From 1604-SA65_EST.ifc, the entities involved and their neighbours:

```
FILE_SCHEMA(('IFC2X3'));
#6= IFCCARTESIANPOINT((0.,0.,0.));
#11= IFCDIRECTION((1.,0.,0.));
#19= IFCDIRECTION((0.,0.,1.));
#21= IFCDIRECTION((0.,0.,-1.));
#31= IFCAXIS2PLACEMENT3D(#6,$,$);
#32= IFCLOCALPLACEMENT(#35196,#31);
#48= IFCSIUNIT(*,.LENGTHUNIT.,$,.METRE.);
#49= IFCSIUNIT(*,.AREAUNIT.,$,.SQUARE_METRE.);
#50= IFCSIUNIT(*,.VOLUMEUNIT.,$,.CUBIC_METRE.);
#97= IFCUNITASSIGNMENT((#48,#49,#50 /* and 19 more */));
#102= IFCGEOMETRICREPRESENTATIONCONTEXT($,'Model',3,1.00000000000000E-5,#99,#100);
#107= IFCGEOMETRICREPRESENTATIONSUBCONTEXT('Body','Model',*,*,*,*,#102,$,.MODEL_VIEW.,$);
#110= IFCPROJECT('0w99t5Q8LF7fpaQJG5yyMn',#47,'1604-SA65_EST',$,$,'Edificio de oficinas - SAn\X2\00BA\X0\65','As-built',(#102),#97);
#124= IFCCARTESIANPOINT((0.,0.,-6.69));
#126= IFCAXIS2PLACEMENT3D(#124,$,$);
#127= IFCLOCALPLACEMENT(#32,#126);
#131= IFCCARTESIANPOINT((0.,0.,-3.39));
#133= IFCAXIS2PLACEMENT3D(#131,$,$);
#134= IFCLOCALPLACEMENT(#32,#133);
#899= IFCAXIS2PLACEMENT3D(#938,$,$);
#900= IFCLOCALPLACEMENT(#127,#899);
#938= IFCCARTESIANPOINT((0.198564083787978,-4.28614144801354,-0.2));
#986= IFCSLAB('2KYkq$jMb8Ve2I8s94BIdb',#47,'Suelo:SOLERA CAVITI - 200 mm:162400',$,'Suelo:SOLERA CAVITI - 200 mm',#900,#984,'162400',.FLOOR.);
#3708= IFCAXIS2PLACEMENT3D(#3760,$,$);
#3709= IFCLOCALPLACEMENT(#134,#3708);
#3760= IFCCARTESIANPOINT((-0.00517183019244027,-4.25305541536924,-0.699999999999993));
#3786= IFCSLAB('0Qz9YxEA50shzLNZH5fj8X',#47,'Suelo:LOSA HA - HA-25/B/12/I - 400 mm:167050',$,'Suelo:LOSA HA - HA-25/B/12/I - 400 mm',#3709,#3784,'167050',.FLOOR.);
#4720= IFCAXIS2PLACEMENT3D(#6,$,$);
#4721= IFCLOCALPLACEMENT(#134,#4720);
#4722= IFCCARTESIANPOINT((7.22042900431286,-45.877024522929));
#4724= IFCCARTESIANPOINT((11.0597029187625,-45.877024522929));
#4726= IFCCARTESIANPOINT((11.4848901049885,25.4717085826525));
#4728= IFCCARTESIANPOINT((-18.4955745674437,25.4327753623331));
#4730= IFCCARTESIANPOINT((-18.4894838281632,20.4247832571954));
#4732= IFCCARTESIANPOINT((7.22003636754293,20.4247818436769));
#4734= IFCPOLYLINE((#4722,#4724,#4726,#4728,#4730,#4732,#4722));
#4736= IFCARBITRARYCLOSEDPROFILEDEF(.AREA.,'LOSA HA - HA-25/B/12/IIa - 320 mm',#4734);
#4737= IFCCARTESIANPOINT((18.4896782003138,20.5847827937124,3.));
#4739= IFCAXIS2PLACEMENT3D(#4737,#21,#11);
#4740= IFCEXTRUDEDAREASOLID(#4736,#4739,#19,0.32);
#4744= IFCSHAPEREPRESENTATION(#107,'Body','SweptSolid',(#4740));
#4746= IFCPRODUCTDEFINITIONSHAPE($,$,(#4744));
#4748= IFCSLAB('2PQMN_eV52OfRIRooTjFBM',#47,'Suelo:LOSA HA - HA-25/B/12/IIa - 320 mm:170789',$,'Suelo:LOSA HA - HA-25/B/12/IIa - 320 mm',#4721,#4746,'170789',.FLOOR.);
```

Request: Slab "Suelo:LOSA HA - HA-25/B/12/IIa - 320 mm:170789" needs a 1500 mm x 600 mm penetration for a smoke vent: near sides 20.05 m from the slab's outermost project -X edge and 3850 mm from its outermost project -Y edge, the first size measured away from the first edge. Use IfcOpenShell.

```python
import numpy as np
import ifcopenshell
import ifcopenshell.api.feature
import ifcopenshell.api.geometry
import ifcopenshell.api.root
import ifcopenshell.geom
import ifcopenshell.util.placement
import ifcopenshell.util.representation
import ifcopenshell.util.shape
import ifcopenshell.util.unit

model = ifcopenshell.open("1604-SA65_EST.ifc")
unit_scale = ifcopenshell.util.unit.calculate_unit_scale(model)
settings = ifcopenshell.geom.settings()


def volume(element):
    """Net volume in cubic metres, openings subtracted."""
    shape = ifcopenshell.geom.create_shape(settings, element)
    return ifcopenshell.util.shape.get_volume(shape.geometry)


slab = model.by_guid("2PQMN_eV52OfRIRooTjFBM")
before = volume(slab)

# Extent in the slab's own axes, in metres. The edges named are its -X and -Y sides.
slab_shape = ifcopenshell.geom.create_shape(settings, slab)
vertices = ifcopenshell.util.shape.get_vertices(slab_shape.geometry)
x_min, y_min, bottom = vertices.min(axis=0)
top = vertices[:, 2].max()

opening = ifcopenshell.api.root.create_entity(model, ifc_class="IfcOpeningElement", name="Smoke vent opening")
context = ifcopenshell.util.representation.get_context(model, "Model", "Body", "MODEL_VIEW")
width, depth = 1.5, 0.6
outline = [(0.0, 0.0), (width, 0.0), (width, depth), (0.0, depth), (0.0, 0.0)]
# Overshoot both faces by 50 mm so the cut is clean.
shape = ifcopenshell.api.geometry.add_slab_representation(
    model, context=context, depth=top - bottom + 0.1, polyline=outline
)
ifcopenshell.api.geometry.assign_representation(model, product=opening, representation=shape)

matrix = ifcopenshell.util.placement.get_local_placement(slab.ObjectPlacement)
matrix[:, 3] = matrix @ np.append(np.array([x_min + 20.05, y_min + 3.85, bottom - 0.05]) / unit_scale, 1.0)
ifcopenshell.api.geometry.edit_object_placement(model, product=opening, matrix=matrix, is_si=False)
ifcopenshell.api.feature.add_feature(model, feature=opening, element=slab)

after = volume(slab)

print(f"slab volume {before:.3f} -> {after:.3f} m3")

model.write("1604-SA65_EST-out.ifc")
```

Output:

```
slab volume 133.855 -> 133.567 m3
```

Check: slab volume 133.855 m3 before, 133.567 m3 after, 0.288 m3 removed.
